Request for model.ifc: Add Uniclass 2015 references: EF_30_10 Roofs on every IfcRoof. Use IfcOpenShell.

First a look at what the model holds.

```python
import ifcopenshell

model = ifcopenshell.open("model.ifc")
print(model.schema)
print("classifications:", [c.Name for c in model.by_type("IfcClassification")])
for ifc_class in ("IfcDoor", "IfcRoof", "IfcStair", "IfcWall", "IfcWindow"):
    print(ifc_class, len(model.by_type(ifc_class)))
```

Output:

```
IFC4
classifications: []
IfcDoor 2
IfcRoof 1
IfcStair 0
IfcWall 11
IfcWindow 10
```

```python
import ifcopenshell
import ifcopenshell.api.classification

model = ifcopenshell.open("model.ifc")

system = ifcopenshell.api.classification.add_classification(model, classification="Uniclass 2015")

codes = {
    "IfcRoof": ("EF_30_10", "Roofs"),
}
for ifc_class, (code, name) in codes.items():
    products = model.by_type(ifc_class)
    ifcopenshell.api.classification.add_reference(
        model, products=products, classification=system, identification=code, name=name
    )
    print(code, len(products))

model.write("model_updated.ifc")
```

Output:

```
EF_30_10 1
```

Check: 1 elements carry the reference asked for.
